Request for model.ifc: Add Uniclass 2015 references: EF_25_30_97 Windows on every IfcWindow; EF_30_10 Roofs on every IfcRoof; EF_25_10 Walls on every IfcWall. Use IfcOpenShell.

First a look at what the model holds.

```python
import ifcopenshell

model = ifcopenshell.open("model.ifc")
print(model.schema)
print("classifications:", [c.Name for c in model.by_type("IfcClassification")])
for ifc_class in ("IfcDoor", "IfcRoof", "IfcStair", "IfcWall", "IfcWindow"):
    print(ifc_class, len(model.by_type(ifc_class)))
```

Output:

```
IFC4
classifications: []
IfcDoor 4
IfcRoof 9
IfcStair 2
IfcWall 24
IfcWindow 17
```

```python
import ifcopenshell
import ifcopenshell.api.classification

model = ifcopenshell.open("model.ifc")

system = ifcopenshell.api.classification.add_classification(model, classification="Uniclass 2015")

codes = {
    "IfcWindow": ("EF_25_30_97", "Windows"),
    "IfcRoof": ("EF_30_10", "Roofs"),
    "IfcWall": ("EF_25_10", "Walls"),
}
for ifc_class, (code, name) in codes.items():
    products = model.by_type(ifc_class)
    ifcopenshell.api.classification.add_reference(
        model, products=products, classification=system, identification=code, name=name
    )
    print(code, len(products))

model.write("model_updated.ifc")
```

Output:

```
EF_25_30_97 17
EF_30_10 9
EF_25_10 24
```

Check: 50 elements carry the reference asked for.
